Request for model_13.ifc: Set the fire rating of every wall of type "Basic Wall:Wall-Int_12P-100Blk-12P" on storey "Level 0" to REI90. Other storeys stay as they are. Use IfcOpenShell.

First a look at what the model holds.

```python
import ifcopenshell
import ifcopenshell.util.element

model = ifcopenshell.open("model_13.ifc")
print(model.schema)
storey = next(s for s in model.by_type("IfcBuildingStorey") if s.Name == "Level 0")
walls = [e for e in ifcopenshell.util.element.get_decomposition(storey) if e.is_a("IfcWall")]
seen = {}
for e in walls:
    element_type = ifcopenshell.util.element.get_type(e)
    key = (element_type.Name if element_type != e and element_type else None, ifcopenshell.util.element.get_pset(e, "Pset_WallCommon", "FireRating"))
    seen[key] = seen.get(key, 0) + 1
for (name, value), count in sorted(seen.items(), key=str):
    print(count, "x", name, "|", value)
```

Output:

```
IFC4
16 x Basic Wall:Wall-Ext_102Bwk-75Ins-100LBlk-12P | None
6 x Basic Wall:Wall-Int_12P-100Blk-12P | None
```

```python
import ifcopenshell
import ifcopenshell.api.pset
import ifcopenshell.util.element

model = ifcopenshell.open("model_13.ifc")

storey = next(s for s in model.by_type("IfcBuildingStorey") if s.Name == "Level 0")
walls = [e for e in ifcopenshell.util.element.get_decomposition(storey) if e.is_a("IfcWall")]

count = 0
for e in walls:
    element_type = ifcopenshell.util.element.get_type(e)
    if element_type in (None, e) or element_type.Name != "Basic Wall:Wall-Int_12P-100Blk-12P":
        continue
    # add_pset returns the element's existing set when there is one.
    pset = ifcopenshell.api.pset.add_pset(model, product=e, name="Pset_WallCommon")
    ifcopenshell.api.pset.edit_pset(model, pset=pset, properties={"FireRating": "REI90"})
    count += 1

print(count, "walls updated")

model.write("model_13_updated.ifc")
```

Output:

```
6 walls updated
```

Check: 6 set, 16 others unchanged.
